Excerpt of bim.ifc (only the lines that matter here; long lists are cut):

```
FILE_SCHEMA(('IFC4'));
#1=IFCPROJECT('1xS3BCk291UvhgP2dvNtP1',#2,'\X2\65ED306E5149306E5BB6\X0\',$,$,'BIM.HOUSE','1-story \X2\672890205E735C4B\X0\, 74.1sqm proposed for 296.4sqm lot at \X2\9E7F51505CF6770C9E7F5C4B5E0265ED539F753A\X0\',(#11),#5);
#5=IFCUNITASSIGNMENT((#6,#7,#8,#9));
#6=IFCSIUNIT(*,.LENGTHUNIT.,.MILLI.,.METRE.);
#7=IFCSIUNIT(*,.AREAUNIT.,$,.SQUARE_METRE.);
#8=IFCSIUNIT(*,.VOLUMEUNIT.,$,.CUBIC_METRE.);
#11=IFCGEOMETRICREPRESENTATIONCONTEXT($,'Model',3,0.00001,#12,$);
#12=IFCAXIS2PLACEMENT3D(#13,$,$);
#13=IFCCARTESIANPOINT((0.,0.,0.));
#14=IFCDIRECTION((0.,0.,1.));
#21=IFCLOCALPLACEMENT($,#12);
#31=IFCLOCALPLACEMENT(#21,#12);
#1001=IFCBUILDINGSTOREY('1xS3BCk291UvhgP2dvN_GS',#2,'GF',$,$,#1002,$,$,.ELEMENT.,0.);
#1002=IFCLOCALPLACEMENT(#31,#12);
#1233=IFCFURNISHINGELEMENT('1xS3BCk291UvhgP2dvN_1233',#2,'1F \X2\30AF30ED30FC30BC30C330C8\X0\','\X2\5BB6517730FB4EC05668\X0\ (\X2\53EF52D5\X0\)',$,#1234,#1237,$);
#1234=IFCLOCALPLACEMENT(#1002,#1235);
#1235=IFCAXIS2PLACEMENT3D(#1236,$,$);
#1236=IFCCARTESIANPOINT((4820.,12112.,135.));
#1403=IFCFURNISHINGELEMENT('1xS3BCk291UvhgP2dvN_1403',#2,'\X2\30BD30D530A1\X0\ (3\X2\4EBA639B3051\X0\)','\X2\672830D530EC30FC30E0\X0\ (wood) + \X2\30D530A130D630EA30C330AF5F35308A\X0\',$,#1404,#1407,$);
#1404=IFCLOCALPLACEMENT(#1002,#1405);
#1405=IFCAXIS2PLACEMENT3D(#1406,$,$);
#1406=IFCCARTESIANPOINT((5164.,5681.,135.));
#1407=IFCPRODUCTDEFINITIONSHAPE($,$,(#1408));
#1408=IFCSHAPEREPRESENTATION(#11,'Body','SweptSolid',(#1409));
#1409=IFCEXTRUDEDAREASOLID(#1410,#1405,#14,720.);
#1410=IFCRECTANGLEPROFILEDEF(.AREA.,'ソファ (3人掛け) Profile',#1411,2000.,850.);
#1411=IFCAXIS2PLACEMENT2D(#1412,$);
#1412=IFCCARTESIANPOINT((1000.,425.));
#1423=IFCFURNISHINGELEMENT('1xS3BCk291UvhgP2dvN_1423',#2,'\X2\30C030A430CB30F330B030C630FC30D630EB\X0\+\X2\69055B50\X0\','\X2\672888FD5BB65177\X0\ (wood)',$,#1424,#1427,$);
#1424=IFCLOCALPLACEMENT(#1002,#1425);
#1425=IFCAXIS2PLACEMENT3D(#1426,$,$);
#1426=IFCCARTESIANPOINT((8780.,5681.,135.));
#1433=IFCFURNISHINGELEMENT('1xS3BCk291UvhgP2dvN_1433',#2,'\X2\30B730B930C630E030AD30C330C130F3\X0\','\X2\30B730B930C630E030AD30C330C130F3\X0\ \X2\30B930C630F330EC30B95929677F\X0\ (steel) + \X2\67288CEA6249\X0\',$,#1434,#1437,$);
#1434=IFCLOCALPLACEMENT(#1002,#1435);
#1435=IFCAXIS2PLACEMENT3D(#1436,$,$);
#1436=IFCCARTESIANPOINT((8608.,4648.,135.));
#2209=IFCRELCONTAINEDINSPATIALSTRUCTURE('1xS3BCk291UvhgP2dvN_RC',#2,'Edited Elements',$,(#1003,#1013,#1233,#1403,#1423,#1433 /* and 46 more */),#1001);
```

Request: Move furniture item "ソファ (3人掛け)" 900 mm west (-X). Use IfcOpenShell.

```python
import ifcopenshell
import ifcopenshell.api.geometry
import ifcopenshell.util.placement
import ifcopenshell.util.unit

model = ifcopenshell.open("bim.ifc")
unit_scale = ifcopenshell.util.unit.calculate_unit_scale(model)

item = model.by_guid("1xS3BCk291UvhgP2dvN_1403")
matrix = ifcopenshell.util.placement.get_local_placement(item.ObjectPlacement)
matrix[0, 3] -= 0.9 / unit_scale
ifcopenshell.api.geometry.edit_object_placement(model, product=item, matrix=matrix, is_si=False)

print(ifcopenshell.util.placement.get_local_placement(item.ObjectPlacement).round(3) + 0.0)

model.write("bim_rev.ifc")
```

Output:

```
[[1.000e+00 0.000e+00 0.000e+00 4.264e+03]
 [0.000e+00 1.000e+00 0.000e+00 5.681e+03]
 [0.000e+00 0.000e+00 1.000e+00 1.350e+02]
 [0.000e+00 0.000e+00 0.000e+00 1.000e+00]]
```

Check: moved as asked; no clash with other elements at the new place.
